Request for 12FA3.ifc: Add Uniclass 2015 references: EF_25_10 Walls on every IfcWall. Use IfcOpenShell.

First a look at what the model holds.

```python
import ifcopenshell

model = ifcopenshell.open("12FA3.ifc")
print(model.schema)
print("classifications:", [c.Name for c in model.by_type("IfcClassification")])
for ifc_class in ("IfcDoor", "IfcRoof", "IfcStair", "IfcWall", "IfcWindow"):
    print(ifc_class, len(model.by_type(ifc_class)))
```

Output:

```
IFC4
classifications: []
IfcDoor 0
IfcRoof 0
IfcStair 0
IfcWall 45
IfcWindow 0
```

```python
import ifcopenshell
import ifcopenshell.api.classification

model = ifcopenshell.open("12FA3.ifc")

system = ifcopenshell.api.classification.add_classification(model, classification="Uniclass 2015")

codes = {
    "IfcWall": ("EF_25_10", "Walls"),
}
for ifc_class, (code, name) in codes.items():
    products = model.by_type(ifc_class)
    ifcopenshell.api.classification.add_reference(
        model, products=products, classification=system, identification=code, name=name
    )
    print(code, len(products))

model.write("12FA3_edited.ifc")
```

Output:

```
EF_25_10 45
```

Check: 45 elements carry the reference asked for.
